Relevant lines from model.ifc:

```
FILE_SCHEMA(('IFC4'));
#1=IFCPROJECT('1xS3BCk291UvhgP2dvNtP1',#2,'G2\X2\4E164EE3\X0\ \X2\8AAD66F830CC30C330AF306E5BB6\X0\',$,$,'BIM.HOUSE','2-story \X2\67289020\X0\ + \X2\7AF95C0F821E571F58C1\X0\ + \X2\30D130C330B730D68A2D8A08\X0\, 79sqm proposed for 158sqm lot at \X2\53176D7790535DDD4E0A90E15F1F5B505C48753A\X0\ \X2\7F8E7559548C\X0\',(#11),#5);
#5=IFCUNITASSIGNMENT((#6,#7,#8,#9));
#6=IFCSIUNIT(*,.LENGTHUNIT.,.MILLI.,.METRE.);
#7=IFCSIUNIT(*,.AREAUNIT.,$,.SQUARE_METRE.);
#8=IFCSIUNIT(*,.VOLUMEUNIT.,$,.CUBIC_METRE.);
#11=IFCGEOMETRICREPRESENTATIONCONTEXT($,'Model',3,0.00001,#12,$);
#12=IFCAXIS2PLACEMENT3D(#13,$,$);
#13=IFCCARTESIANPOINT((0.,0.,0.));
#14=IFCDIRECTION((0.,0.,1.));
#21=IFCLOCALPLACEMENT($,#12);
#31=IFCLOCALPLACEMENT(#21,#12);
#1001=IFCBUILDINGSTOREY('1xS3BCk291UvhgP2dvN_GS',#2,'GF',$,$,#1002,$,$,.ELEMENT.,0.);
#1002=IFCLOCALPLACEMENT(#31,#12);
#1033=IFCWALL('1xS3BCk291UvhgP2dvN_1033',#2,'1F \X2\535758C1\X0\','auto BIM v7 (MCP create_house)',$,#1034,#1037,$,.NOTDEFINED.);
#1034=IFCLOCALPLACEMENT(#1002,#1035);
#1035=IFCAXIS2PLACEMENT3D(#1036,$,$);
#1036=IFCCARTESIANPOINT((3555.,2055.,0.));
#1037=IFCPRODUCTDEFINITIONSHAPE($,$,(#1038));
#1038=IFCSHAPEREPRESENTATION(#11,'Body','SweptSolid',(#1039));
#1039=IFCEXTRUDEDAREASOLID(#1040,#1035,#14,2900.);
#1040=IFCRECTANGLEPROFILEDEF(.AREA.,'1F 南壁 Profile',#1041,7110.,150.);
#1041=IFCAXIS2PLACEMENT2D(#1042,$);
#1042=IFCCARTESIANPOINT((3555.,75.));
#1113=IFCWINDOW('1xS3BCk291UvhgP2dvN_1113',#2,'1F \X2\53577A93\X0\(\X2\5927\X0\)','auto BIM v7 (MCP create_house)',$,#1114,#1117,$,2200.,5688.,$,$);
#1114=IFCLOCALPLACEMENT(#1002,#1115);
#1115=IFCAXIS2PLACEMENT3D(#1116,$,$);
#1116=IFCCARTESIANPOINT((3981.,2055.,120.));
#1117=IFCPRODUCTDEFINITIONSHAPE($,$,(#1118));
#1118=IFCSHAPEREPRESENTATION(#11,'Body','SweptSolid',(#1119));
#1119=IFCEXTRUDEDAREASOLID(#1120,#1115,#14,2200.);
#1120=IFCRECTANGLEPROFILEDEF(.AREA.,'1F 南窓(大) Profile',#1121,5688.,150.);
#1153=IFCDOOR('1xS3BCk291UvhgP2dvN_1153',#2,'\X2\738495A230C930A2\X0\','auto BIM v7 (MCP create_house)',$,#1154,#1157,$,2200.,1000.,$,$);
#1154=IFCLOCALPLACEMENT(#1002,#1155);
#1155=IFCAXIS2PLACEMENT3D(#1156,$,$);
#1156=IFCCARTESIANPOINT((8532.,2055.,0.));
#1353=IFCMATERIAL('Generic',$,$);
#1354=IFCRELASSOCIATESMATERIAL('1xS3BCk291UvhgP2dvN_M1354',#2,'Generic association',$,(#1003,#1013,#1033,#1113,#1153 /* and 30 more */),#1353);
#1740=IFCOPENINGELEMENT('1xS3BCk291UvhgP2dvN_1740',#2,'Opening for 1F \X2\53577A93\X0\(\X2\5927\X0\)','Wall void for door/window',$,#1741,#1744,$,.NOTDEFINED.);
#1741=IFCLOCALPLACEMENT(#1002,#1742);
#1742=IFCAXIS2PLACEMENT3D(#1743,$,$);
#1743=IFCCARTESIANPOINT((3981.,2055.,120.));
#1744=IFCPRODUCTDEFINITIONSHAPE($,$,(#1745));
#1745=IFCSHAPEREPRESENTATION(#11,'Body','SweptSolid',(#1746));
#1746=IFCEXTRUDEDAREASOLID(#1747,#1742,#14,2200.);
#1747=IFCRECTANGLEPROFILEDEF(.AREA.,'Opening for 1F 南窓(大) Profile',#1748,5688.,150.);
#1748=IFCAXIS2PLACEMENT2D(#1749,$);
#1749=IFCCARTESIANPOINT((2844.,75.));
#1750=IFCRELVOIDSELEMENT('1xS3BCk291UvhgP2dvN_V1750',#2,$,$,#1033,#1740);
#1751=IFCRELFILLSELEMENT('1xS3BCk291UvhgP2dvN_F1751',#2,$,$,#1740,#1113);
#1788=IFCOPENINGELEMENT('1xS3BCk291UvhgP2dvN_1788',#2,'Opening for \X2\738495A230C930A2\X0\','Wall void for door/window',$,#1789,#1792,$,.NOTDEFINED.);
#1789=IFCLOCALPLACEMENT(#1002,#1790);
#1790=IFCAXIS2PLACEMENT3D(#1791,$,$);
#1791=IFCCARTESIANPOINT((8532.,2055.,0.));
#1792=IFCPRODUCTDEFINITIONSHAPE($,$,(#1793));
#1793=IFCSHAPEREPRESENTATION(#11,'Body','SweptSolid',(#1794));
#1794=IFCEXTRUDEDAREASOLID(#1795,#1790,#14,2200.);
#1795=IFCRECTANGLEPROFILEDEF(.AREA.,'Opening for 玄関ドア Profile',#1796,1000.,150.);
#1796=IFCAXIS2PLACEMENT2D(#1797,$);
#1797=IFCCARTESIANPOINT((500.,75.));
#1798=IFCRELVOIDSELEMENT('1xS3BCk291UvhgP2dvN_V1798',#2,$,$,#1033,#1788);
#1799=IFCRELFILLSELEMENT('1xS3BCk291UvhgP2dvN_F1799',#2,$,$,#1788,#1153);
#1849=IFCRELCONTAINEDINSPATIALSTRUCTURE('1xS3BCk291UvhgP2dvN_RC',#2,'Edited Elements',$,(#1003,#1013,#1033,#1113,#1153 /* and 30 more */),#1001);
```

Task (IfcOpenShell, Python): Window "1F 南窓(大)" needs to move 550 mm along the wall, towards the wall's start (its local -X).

```python
import ifcopenshell
import ifcopenshell.api.geometry
import ifcopenshell.util.placement

model = ifcopenshell.open("model.ifc")

window = model.by_guid("1xS3BCk291UvhgP2dvN_1113")
opening = window.FillsVoids[0].RelatingOpeningElement
wall = opening.VoidsElements[0].RelatingBuildingElement

wall_matrix = ifcopenshell.util.placement.get_local_placement(wall.ObjectPlacement)
shift = wall_matrix[:3, 0] * -550.0
before = ifcopenshell.util.placement.get_local_placement(window.ObjectPlacement)[:3, 3].copy()

# The window is not placed relative to its opening, so move both.
for product in (opening, window):
    matrix = ifcopenshell.util.placement.get_local_placement(product.ObjectPlacement)
    matrix[:3, 3] += shift
    ifcopenshell.api.geometry.edit_object_placement(model, product=product, matrix=matrix, is_si=False)

after = ifcopenshell.util.placement.get_local_placement(window.ObjectPlacement)[:3, 3]
print("window moved by", (after - before).round(3) + 0.0)

model.write("model-out.ifc")
```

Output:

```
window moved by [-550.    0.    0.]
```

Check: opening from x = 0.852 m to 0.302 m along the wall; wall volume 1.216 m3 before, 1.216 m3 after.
